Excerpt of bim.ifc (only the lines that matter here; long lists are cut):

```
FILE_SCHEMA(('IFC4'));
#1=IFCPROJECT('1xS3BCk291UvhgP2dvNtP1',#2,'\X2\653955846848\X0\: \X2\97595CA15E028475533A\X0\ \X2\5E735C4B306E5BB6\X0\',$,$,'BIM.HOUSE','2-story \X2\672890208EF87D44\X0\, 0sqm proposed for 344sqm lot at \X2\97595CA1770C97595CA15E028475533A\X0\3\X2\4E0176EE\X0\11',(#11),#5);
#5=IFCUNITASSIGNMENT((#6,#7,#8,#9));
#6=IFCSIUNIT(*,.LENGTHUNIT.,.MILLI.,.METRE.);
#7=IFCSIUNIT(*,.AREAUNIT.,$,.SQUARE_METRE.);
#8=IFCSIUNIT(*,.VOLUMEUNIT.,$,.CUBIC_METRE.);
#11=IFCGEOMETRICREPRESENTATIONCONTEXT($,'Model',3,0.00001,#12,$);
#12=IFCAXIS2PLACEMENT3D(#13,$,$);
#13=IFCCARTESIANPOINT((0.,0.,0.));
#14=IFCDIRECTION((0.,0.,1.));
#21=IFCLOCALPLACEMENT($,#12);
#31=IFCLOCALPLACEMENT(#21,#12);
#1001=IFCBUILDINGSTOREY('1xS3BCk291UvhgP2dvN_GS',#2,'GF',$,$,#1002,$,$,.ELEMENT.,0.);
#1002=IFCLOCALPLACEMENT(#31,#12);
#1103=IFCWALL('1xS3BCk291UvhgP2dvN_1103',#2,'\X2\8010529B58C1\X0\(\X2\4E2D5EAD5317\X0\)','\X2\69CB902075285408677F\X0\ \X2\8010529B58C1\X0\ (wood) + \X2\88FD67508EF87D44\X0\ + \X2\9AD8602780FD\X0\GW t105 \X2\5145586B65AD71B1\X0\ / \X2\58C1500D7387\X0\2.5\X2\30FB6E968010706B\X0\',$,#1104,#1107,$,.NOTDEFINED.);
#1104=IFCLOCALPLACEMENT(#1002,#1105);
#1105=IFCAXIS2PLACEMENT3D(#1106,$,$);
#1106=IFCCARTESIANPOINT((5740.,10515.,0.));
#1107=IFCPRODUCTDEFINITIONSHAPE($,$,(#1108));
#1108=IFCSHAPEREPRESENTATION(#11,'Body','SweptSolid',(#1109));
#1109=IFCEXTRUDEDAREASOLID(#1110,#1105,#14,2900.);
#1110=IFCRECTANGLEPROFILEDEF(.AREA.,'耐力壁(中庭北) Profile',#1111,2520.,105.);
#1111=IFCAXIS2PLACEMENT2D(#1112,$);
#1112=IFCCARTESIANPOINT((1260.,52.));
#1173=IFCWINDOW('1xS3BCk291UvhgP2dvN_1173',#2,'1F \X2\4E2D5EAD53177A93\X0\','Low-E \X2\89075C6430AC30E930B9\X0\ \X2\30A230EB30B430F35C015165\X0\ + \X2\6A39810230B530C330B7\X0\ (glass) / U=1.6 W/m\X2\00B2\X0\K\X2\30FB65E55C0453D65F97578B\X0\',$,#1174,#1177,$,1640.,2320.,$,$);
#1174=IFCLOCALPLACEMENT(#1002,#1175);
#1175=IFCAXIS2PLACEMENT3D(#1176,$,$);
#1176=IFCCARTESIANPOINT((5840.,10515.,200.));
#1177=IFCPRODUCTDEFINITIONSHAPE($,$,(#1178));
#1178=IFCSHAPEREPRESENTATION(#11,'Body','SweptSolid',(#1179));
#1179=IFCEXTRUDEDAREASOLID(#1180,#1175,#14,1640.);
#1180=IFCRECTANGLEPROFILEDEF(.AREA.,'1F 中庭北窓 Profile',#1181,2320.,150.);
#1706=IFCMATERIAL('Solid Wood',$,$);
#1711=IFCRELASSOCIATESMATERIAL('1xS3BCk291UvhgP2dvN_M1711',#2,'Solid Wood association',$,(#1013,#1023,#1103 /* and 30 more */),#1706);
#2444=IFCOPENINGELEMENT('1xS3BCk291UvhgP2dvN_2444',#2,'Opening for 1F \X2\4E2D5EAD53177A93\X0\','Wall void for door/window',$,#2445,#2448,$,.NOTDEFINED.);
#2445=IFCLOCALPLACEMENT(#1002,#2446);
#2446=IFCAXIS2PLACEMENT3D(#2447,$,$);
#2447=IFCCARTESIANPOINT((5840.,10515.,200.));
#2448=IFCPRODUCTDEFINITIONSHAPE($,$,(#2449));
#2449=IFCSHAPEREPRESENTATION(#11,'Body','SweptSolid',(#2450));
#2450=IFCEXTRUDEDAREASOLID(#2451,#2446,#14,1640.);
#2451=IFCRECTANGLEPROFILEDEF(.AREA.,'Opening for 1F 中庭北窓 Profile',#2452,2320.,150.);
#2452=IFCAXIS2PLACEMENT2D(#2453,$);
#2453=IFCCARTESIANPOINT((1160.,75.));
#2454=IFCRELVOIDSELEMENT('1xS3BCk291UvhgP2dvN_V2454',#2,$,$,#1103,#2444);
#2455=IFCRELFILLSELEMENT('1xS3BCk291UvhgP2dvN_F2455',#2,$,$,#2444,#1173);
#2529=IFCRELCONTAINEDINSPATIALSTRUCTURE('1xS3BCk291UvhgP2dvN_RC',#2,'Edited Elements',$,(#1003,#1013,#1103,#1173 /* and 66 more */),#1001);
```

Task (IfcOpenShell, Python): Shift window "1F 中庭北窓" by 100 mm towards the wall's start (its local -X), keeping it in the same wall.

```python
import ifcopenshell
import ifcopenshell.api.geometry
import ifcopenshell.util.placement
import ifcopenshell.util.unit

model = ifcopenshell.open("bim.ifc")
unit_scale = ifcopenshell.util.unit.calculate_unit_scale(model)

window = model.by_id(1173)
opening = window.FillsVoids[0].RelatingOpeningElement
wall = opening.VoidsElements[0].RelatingBuildingElement

wall_matrix = ifcopenshell.util.placement.get_local_placement(wall.ObjectPlacement)
shift = wall_matrix[:3, 0] * -0.1 / unit_scale
before = ifcopenshell.util.placement.get_local_placement(window.ObjectPlacement)[:3, 3].copy()

# The window is not placed relative to its opening, so move both.
for product in (opening, window):
    matrix = ifcopenshell.util.placement.get_local_placement(product.ObjectPlacement)
    matrix[:3, 3] += shift
    ifcopenshell.api.geometry.edit_object_placement(model, product=product, matrix=matrix, is_si=False)

after = ifcopenshell.util.placement.get_local_placement(window.ObjectPlacement)[:3, 3]
print("window moved by", (after - before).round(3) + 0.0)

model.write("bim-out.ifc")
```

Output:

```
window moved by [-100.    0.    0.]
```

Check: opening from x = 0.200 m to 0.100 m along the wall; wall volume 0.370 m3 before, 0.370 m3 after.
